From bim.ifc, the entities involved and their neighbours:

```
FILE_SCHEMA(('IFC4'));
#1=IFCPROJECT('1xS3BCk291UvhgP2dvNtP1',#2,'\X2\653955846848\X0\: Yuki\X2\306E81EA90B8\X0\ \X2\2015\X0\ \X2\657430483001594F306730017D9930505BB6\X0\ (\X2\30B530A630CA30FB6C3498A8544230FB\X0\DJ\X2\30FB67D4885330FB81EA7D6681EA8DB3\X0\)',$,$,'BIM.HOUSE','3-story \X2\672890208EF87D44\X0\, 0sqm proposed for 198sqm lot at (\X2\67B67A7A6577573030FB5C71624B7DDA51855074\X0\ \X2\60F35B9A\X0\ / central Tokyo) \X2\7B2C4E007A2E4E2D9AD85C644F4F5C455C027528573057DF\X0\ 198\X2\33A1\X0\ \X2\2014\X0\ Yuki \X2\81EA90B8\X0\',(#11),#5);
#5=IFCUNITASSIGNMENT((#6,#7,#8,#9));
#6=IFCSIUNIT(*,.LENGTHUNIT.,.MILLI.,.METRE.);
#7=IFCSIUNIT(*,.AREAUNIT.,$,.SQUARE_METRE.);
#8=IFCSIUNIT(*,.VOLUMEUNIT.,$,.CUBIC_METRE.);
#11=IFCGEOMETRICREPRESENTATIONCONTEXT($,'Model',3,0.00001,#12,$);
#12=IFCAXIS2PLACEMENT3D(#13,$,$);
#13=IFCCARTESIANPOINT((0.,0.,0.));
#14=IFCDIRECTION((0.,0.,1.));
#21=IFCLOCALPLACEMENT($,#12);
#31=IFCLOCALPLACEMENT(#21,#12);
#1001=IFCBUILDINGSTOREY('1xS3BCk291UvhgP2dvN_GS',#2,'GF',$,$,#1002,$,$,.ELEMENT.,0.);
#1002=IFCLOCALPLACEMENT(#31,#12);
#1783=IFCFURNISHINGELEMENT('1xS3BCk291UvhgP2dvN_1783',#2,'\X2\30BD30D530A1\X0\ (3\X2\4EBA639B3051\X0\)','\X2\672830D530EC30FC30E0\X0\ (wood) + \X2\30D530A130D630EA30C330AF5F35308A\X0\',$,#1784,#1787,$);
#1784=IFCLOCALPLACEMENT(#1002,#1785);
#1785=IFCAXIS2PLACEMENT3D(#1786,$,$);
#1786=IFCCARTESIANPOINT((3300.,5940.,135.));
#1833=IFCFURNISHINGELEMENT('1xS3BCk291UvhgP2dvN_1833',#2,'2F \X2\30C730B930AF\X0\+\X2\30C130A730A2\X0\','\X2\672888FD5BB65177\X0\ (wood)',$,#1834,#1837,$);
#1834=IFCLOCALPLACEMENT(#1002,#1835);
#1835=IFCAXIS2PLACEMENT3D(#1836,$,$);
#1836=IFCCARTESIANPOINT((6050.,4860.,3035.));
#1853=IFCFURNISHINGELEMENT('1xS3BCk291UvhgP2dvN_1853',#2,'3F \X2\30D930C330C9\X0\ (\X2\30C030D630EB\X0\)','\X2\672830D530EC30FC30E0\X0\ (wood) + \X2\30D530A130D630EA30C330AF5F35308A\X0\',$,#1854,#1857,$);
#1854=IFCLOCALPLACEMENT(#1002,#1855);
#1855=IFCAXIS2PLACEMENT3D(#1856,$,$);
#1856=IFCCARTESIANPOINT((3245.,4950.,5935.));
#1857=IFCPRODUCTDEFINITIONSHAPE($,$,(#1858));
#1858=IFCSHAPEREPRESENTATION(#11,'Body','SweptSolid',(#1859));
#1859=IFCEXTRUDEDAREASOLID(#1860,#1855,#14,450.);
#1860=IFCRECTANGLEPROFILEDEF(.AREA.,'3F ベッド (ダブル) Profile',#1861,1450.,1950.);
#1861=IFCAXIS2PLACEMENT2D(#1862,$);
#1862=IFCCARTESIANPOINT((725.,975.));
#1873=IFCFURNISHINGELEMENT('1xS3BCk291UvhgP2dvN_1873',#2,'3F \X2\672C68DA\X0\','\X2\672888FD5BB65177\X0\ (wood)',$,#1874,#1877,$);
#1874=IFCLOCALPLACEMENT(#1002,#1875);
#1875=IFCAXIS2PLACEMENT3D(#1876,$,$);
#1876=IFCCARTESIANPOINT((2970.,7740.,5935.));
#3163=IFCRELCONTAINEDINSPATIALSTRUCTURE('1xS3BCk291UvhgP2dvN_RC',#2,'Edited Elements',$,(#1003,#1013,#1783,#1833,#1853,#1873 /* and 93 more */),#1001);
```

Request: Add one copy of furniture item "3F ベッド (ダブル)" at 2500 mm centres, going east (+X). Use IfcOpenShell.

```python
import numpy as np
import ifcopenshell
import ifcopenshell.api.geometry
import ifcopenshell.api.root
import ifcopenshell.util.element
import ifcopenshell.util.placement
import ifcopenshell.util.unit

model = ifcopenshell.open("bim.ifc")
unit_scale = ifcopenshell.util.unit.calculate_unit_scale(model)


def reuse_history(source, copy):
    """copy_class also copies each property set's owner history, people and application; keep the originals."""
    for rel in copy.IsDefinedBy:
        if rel.is_a("IfcRelDefinesByProperties") and (history := rel.RelatingPropertyDefinition.OwnerHistory):
            rel.RelatingPropertyDefinition.OwnerHistory = source.OwnerHistory
            ifcopenshell.util.element.remove_deep2(model, history)


source = model.by_guid("1xS3BCk291UvhgP2dvN_1853")
base = ifcopenshell.util.placement.get_local_placement(source.ObjectPlacement)
step = np.array([1.0, 0.0, 0.0]) * 2.5 / unit_scale

for i in range(1, 2):
    copy = ifcopenshell.api.root.copy_class(model, product=source)
    copy.Representation = ifcopenshell.util.element.copy_deep(
        model, source.Representation, exclude=["IfcGeometricRepresentationContext", "IfcRepresentationMap"]
    )
    reuse_history(source, copy)
    matrix = base.copy()
    matrix[:3, 3] += i * step
    print("added at", matrix[:3, 3].round(3) + 0.0)
    ifcopenshell.api.geometry.edit_object_placement(model, product=copy, matrix=matrix, is_si=False)

model.write("bim_edited.ifc")
```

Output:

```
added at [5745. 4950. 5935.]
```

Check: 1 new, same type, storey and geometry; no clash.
